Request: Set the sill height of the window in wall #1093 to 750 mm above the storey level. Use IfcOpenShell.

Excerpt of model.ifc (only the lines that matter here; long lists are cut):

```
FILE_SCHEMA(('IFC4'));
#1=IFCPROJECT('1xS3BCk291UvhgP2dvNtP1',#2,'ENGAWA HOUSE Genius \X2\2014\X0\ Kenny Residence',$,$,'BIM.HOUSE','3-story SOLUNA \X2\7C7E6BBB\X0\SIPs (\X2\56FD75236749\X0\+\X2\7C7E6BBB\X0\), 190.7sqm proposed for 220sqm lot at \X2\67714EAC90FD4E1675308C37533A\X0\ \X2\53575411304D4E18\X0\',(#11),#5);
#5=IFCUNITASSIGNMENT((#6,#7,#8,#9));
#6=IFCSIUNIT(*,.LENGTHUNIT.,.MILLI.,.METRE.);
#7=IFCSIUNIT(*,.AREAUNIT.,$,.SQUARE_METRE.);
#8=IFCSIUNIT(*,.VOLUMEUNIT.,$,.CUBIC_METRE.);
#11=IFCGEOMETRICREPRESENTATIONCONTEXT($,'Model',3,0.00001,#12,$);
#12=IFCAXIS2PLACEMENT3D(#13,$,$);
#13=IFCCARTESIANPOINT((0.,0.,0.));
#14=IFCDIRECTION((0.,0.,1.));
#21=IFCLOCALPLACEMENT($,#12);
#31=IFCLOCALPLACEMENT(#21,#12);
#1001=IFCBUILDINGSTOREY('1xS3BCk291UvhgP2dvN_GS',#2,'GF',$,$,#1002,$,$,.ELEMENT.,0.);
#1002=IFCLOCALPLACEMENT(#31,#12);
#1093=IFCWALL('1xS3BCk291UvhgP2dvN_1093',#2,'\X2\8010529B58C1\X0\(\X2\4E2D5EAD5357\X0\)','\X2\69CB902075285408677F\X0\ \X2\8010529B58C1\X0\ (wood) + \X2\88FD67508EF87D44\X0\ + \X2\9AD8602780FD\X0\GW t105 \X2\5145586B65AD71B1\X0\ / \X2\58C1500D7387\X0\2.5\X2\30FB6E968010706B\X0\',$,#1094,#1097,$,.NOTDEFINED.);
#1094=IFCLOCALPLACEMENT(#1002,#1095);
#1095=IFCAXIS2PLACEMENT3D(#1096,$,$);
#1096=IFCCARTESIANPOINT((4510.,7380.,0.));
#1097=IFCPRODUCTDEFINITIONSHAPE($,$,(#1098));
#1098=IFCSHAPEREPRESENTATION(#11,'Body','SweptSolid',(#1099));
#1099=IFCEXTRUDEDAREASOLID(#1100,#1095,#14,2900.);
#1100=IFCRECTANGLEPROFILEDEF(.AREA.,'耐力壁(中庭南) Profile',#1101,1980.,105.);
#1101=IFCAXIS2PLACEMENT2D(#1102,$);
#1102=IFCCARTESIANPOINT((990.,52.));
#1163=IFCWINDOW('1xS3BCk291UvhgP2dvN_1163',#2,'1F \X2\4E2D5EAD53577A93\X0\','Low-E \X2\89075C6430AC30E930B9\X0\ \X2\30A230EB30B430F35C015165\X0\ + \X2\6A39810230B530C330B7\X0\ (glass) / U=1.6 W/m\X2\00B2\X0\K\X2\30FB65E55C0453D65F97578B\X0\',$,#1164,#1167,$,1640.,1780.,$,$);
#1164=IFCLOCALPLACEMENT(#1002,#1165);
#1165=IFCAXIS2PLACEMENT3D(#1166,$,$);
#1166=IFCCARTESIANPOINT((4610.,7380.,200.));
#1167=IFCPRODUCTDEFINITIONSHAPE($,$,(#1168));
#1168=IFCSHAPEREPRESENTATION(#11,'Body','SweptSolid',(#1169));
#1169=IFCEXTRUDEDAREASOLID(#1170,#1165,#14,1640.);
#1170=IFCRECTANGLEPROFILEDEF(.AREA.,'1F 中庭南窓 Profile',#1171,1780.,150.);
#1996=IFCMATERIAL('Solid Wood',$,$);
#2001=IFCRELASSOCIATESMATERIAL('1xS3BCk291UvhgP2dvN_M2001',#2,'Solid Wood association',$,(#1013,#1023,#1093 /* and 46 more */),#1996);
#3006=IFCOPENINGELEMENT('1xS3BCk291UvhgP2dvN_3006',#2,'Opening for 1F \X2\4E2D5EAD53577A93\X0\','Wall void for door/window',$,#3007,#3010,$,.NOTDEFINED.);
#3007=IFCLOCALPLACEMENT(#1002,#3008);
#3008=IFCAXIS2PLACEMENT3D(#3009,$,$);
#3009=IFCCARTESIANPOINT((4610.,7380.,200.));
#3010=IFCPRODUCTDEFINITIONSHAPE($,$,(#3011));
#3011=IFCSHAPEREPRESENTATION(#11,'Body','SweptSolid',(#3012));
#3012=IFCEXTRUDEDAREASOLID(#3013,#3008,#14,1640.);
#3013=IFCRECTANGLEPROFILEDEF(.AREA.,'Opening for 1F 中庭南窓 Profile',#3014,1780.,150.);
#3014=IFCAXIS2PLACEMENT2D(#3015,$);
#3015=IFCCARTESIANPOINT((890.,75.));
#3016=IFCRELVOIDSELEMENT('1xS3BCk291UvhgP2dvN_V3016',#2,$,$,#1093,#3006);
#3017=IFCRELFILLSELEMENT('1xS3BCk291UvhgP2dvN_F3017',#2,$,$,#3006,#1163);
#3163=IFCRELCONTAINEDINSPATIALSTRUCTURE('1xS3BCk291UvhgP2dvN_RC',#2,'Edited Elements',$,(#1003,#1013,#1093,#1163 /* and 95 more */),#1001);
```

```python
import numpy as np
import ifcopenshell
import ifcopenshell.api.geometry
import ifcopenshell.geom
import ifcopenshell.util.element
import ifcopenshell.util.placement
import ifcopenshell.util.shape
import ifcopenshell.util.unit

model = ifcopenshell.open("model.ifc")
unit_scale = ifcopenshell.util.unit.calculate_unit_scale(model)

window = model.by_id(1163)
opening = window.FillsVoids[0].RelatingOpeningElement
storey = ifcopenshell.util.element.get_container(window, ifc_class="IfcBuildingStorey")
level = ifcopenshell.util.placement.get_local_placement(storey.ObjectPlacement)[2, 3]

# The opening's origin need not be at the sill, so measure its lowest point.
shape = ifcopenshell.geom.create_shape(ifcopenshell.geom.settings(), opening)
bottom = ifcopenshell.util.shape.get_shape_bottom_elevation(shape, shape.geometry) / unit_scale
dz = level + 750.0 - bottom

shift = np.array([0.0, 0.0, dz])
# The window is not placed relative to its opening, so move both.
for product in (opening, window):
    matrix = ifcopenshell.util.placement.get_local_placement(product.ObjectPlacement)
    matrix[:3, 3] += shift
    ifcopenshell.api.geometry.edit_object_placement(model, product=product, matrix=matrix, is_si=False)

print(f"moved by {dz * unit_scale:+.3f} m")

model.write("model_edited.ifc")
```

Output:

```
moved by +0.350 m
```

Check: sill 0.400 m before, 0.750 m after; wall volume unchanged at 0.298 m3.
